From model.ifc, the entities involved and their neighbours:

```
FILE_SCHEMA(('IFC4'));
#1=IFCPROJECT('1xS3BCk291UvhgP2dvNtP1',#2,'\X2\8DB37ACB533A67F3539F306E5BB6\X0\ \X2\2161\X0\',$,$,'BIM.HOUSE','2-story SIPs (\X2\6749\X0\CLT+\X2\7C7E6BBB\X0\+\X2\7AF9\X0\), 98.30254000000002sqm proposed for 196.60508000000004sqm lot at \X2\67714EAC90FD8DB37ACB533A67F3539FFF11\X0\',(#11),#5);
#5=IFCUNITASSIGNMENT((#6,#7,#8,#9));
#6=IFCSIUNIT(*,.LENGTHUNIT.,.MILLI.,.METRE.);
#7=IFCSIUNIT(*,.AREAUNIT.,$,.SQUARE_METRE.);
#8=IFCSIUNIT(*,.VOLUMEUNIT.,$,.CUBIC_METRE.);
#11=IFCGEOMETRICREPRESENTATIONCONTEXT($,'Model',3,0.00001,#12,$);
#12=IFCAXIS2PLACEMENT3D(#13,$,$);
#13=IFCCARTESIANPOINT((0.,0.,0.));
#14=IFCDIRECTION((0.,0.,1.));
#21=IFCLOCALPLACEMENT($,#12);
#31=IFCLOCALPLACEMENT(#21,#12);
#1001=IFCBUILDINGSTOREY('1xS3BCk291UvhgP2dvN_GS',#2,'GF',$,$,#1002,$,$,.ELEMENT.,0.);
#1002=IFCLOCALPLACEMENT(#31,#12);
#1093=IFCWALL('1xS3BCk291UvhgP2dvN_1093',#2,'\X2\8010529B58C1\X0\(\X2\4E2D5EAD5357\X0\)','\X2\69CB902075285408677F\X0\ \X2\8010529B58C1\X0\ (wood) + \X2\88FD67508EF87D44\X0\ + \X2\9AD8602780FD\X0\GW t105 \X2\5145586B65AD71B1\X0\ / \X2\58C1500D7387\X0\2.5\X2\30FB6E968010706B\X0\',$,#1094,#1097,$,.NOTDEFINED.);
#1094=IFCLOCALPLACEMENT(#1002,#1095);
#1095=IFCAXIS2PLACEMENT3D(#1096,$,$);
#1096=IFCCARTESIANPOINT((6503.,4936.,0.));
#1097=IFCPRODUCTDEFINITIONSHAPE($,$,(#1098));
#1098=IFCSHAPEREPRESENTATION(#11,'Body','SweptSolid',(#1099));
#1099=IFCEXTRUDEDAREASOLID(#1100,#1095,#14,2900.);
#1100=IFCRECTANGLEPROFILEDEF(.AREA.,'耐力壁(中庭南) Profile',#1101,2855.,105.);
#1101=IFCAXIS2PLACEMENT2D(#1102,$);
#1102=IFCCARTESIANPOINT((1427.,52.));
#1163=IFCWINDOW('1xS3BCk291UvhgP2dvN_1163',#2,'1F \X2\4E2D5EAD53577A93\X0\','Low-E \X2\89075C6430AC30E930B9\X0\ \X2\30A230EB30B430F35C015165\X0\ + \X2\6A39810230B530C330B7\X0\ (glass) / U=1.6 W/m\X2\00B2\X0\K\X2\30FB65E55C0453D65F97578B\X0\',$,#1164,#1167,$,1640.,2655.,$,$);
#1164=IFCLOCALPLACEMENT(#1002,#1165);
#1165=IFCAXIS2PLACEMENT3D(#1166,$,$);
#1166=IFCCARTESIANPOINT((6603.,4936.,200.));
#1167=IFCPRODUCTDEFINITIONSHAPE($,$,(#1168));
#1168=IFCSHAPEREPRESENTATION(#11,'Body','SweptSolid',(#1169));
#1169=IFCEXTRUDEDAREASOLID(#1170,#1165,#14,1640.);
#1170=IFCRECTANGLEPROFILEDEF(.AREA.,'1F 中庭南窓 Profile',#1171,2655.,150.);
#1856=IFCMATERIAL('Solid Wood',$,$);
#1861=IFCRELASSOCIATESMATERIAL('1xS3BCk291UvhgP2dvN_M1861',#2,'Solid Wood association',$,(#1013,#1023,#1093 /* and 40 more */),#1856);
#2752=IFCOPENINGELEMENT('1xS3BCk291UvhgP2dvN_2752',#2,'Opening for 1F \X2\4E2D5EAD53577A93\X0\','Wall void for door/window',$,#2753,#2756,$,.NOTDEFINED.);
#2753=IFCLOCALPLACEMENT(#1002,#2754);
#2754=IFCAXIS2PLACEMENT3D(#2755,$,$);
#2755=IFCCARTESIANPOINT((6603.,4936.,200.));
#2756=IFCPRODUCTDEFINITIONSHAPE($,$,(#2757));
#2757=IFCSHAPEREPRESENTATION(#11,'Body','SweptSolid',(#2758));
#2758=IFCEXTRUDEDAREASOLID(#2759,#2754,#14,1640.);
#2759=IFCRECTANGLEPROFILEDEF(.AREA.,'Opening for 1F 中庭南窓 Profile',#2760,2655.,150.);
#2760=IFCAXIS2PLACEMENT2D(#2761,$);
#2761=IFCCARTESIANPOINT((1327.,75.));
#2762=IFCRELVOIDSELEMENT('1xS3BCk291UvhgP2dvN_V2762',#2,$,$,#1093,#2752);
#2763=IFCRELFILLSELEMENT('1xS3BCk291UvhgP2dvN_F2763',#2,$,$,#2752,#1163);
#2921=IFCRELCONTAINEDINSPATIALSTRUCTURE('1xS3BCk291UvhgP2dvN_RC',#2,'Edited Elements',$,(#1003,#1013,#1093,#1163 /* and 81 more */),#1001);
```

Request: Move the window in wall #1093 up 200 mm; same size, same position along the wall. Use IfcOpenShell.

```python
import numpy as np
import ifcopenshell
import ifcopenshell.api.geometry
import ifcopenshell.util.placement
import ifcopenshell.util.unit

model = ifcopenshell.open("model.ifc")
unit_scale = ifcopenshell.util.unit.calculate_unit_scale(model)

window = model.by_id(1163)
opening = window.FillsVoids[0].RelatingOpeningElement
dz = 200.0

shift = np.array([0.0, 0.0, dz])
# The window is not placed relative to its opening, so move both.
for product in (opening, window):
    matrix = ifcopenshell.util.placement.get_local_placement(product.ObjectPlacement)
    matrix[:3, 3] += shift
    ifcopenshell.api.geometry.edit_object_placement(model, product=product, matrix=matrix, is_si=False)

print(f"moved by {dz * unit_scale:+.3f} m")

model.write("model-out.ifc")
```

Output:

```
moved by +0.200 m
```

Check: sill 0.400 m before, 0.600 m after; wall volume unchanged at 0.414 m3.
